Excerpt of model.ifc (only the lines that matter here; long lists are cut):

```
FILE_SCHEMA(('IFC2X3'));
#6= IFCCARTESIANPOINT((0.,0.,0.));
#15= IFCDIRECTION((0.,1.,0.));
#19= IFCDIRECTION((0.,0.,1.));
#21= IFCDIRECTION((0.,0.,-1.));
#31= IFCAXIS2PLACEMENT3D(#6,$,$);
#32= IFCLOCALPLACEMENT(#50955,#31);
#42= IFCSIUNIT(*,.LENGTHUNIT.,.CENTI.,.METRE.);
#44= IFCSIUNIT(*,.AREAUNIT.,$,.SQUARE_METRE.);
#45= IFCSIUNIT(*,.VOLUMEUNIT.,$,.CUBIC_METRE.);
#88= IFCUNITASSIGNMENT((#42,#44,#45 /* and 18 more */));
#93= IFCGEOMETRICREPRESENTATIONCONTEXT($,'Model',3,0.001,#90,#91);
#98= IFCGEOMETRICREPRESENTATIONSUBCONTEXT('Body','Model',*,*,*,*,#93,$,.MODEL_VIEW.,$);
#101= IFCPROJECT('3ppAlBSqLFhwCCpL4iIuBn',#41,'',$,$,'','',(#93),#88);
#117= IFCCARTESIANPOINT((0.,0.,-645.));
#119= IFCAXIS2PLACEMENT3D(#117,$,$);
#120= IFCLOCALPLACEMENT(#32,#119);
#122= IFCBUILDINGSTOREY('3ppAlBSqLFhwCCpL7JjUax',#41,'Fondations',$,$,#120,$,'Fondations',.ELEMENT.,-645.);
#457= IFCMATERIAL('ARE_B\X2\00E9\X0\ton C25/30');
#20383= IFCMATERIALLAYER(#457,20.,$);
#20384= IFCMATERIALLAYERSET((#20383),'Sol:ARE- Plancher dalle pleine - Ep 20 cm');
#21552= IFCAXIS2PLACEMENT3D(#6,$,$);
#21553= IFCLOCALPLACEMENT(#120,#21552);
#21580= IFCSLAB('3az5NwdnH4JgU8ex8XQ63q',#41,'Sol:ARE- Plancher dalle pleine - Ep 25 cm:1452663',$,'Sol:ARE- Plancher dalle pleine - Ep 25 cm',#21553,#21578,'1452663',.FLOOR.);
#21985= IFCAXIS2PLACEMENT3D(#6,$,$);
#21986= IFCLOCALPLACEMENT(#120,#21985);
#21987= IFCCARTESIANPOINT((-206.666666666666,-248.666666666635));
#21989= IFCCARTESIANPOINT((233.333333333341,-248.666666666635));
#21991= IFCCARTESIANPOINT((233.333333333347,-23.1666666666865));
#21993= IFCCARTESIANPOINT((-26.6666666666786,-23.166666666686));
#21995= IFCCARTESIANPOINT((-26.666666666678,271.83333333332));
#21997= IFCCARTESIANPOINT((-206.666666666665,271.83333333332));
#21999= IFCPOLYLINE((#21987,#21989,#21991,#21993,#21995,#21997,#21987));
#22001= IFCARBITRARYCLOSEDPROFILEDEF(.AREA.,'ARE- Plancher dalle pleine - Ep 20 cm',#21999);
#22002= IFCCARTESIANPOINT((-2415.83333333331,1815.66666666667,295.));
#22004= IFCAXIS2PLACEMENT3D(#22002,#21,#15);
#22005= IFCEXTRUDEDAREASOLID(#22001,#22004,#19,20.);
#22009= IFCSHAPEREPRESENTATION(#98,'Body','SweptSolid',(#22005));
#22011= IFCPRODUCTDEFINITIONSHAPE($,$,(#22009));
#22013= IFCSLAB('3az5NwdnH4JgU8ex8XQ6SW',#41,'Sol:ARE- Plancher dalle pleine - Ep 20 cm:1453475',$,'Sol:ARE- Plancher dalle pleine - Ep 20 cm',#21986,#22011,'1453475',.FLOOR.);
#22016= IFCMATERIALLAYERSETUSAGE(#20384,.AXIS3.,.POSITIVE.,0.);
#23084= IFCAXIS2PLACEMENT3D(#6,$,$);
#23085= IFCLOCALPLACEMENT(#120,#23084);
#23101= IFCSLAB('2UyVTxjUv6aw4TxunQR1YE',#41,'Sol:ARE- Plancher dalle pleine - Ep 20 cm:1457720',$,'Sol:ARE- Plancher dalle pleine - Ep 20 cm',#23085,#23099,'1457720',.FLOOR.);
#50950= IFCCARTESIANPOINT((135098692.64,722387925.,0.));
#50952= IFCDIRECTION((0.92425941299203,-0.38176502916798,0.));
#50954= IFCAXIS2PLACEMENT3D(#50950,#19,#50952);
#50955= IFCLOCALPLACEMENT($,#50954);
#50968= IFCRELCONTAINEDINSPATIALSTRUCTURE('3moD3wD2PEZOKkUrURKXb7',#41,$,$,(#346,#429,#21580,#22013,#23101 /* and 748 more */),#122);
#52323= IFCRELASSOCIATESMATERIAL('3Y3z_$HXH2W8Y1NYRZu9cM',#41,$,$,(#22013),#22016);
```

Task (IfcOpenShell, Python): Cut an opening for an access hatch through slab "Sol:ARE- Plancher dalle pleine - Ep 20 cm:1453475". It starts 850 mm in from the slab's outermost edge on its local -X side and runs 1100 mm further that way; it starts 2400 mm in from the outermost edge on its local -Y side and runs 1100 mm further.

```python
import numpy as np
import ifcopenshell
import ifcopenshell.api.feature
import ifcopenshell.api.geometry
import ifcopenshell.api.root
import ifcopenshell.geom
import ifcopenshell.util.placement
import ifcopenshell.util.representation
import ifcopenshell.util.shape
import ifcopenshell.util.unit

model = ifcopenshell.open("model.ifc")
unit_scale = ifcopenshell.util.unit.calculate_unit_scale(model)
settings = ifcopenshell.geom.settings()


def volume(element):
    """Net volume in cubic metres, openings subtracted."""
    shape = ifcopenshell.geom.create_shape(settings, element)
    return ifcopenshell.util.shape.get_volume(shape.geometry)


slab = model.by_guid("3az5NwdnH4JgU8ex8XQ6SW")
before = volume(slab)

# Extent in the slab's own axes, in metres. The edges named are its -X and -Y sides.
slab_shape = ifcopenshell.geom.create_shape(settings, slab)
vertices = ifcopenshell.util.shape.get_vertices(slab_shape.geometry)
x_min, y_min, bottom = vertices.min(axis=0)
top = vertices[:, 2].max()

opening = ifcopenshell.api.root.create_entity(model, ifc_class="IfcOpeningElement", name="Access hatch opening")
context = ifcopenshell.util.representation.get_context(model, "Model", "Body", "MODEL_VIEW")
width, depth = 1.1, 1.1
outline = [(0.0, 0.0), (width, 0.0), (width, depth), (0.0, depth), (0.0, 0.0)]
# Overshoot both faces by 50 mm so the cut is clean.
shape = ifcopenshell.api.geometry.add_slab_representation(
    model, context=context, depth=top - bottom + 0.1, polyline=outline
)
ifcopenshell.api.geometry.assign_representation(model, product=opening, representation=shape)

matrix = ifcopenshell.util.placement.get_local_placement(slab.ObjectPlacement)
matrix[:, 3] = matrix @ np.append(np.array([x_min + 0.85, y_min + 2.4, bottom - 0.05]) / unit_scale, 1.0)
ifcopenshell.api.geometry.edit_object_placement(model, product=opening, matrix=matrix, is_si=False)
ifcopenshell.api.feature.add_feature(model, feature=opening, element=slab)

after = volume(slab)

print(f"slab volume {before:.3f} -> {after:.3f} m3")

model.write("model_rev.ifc")
```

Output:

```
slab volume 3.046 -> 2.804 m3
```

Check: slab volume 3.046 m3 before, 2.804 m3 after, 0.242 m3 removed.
